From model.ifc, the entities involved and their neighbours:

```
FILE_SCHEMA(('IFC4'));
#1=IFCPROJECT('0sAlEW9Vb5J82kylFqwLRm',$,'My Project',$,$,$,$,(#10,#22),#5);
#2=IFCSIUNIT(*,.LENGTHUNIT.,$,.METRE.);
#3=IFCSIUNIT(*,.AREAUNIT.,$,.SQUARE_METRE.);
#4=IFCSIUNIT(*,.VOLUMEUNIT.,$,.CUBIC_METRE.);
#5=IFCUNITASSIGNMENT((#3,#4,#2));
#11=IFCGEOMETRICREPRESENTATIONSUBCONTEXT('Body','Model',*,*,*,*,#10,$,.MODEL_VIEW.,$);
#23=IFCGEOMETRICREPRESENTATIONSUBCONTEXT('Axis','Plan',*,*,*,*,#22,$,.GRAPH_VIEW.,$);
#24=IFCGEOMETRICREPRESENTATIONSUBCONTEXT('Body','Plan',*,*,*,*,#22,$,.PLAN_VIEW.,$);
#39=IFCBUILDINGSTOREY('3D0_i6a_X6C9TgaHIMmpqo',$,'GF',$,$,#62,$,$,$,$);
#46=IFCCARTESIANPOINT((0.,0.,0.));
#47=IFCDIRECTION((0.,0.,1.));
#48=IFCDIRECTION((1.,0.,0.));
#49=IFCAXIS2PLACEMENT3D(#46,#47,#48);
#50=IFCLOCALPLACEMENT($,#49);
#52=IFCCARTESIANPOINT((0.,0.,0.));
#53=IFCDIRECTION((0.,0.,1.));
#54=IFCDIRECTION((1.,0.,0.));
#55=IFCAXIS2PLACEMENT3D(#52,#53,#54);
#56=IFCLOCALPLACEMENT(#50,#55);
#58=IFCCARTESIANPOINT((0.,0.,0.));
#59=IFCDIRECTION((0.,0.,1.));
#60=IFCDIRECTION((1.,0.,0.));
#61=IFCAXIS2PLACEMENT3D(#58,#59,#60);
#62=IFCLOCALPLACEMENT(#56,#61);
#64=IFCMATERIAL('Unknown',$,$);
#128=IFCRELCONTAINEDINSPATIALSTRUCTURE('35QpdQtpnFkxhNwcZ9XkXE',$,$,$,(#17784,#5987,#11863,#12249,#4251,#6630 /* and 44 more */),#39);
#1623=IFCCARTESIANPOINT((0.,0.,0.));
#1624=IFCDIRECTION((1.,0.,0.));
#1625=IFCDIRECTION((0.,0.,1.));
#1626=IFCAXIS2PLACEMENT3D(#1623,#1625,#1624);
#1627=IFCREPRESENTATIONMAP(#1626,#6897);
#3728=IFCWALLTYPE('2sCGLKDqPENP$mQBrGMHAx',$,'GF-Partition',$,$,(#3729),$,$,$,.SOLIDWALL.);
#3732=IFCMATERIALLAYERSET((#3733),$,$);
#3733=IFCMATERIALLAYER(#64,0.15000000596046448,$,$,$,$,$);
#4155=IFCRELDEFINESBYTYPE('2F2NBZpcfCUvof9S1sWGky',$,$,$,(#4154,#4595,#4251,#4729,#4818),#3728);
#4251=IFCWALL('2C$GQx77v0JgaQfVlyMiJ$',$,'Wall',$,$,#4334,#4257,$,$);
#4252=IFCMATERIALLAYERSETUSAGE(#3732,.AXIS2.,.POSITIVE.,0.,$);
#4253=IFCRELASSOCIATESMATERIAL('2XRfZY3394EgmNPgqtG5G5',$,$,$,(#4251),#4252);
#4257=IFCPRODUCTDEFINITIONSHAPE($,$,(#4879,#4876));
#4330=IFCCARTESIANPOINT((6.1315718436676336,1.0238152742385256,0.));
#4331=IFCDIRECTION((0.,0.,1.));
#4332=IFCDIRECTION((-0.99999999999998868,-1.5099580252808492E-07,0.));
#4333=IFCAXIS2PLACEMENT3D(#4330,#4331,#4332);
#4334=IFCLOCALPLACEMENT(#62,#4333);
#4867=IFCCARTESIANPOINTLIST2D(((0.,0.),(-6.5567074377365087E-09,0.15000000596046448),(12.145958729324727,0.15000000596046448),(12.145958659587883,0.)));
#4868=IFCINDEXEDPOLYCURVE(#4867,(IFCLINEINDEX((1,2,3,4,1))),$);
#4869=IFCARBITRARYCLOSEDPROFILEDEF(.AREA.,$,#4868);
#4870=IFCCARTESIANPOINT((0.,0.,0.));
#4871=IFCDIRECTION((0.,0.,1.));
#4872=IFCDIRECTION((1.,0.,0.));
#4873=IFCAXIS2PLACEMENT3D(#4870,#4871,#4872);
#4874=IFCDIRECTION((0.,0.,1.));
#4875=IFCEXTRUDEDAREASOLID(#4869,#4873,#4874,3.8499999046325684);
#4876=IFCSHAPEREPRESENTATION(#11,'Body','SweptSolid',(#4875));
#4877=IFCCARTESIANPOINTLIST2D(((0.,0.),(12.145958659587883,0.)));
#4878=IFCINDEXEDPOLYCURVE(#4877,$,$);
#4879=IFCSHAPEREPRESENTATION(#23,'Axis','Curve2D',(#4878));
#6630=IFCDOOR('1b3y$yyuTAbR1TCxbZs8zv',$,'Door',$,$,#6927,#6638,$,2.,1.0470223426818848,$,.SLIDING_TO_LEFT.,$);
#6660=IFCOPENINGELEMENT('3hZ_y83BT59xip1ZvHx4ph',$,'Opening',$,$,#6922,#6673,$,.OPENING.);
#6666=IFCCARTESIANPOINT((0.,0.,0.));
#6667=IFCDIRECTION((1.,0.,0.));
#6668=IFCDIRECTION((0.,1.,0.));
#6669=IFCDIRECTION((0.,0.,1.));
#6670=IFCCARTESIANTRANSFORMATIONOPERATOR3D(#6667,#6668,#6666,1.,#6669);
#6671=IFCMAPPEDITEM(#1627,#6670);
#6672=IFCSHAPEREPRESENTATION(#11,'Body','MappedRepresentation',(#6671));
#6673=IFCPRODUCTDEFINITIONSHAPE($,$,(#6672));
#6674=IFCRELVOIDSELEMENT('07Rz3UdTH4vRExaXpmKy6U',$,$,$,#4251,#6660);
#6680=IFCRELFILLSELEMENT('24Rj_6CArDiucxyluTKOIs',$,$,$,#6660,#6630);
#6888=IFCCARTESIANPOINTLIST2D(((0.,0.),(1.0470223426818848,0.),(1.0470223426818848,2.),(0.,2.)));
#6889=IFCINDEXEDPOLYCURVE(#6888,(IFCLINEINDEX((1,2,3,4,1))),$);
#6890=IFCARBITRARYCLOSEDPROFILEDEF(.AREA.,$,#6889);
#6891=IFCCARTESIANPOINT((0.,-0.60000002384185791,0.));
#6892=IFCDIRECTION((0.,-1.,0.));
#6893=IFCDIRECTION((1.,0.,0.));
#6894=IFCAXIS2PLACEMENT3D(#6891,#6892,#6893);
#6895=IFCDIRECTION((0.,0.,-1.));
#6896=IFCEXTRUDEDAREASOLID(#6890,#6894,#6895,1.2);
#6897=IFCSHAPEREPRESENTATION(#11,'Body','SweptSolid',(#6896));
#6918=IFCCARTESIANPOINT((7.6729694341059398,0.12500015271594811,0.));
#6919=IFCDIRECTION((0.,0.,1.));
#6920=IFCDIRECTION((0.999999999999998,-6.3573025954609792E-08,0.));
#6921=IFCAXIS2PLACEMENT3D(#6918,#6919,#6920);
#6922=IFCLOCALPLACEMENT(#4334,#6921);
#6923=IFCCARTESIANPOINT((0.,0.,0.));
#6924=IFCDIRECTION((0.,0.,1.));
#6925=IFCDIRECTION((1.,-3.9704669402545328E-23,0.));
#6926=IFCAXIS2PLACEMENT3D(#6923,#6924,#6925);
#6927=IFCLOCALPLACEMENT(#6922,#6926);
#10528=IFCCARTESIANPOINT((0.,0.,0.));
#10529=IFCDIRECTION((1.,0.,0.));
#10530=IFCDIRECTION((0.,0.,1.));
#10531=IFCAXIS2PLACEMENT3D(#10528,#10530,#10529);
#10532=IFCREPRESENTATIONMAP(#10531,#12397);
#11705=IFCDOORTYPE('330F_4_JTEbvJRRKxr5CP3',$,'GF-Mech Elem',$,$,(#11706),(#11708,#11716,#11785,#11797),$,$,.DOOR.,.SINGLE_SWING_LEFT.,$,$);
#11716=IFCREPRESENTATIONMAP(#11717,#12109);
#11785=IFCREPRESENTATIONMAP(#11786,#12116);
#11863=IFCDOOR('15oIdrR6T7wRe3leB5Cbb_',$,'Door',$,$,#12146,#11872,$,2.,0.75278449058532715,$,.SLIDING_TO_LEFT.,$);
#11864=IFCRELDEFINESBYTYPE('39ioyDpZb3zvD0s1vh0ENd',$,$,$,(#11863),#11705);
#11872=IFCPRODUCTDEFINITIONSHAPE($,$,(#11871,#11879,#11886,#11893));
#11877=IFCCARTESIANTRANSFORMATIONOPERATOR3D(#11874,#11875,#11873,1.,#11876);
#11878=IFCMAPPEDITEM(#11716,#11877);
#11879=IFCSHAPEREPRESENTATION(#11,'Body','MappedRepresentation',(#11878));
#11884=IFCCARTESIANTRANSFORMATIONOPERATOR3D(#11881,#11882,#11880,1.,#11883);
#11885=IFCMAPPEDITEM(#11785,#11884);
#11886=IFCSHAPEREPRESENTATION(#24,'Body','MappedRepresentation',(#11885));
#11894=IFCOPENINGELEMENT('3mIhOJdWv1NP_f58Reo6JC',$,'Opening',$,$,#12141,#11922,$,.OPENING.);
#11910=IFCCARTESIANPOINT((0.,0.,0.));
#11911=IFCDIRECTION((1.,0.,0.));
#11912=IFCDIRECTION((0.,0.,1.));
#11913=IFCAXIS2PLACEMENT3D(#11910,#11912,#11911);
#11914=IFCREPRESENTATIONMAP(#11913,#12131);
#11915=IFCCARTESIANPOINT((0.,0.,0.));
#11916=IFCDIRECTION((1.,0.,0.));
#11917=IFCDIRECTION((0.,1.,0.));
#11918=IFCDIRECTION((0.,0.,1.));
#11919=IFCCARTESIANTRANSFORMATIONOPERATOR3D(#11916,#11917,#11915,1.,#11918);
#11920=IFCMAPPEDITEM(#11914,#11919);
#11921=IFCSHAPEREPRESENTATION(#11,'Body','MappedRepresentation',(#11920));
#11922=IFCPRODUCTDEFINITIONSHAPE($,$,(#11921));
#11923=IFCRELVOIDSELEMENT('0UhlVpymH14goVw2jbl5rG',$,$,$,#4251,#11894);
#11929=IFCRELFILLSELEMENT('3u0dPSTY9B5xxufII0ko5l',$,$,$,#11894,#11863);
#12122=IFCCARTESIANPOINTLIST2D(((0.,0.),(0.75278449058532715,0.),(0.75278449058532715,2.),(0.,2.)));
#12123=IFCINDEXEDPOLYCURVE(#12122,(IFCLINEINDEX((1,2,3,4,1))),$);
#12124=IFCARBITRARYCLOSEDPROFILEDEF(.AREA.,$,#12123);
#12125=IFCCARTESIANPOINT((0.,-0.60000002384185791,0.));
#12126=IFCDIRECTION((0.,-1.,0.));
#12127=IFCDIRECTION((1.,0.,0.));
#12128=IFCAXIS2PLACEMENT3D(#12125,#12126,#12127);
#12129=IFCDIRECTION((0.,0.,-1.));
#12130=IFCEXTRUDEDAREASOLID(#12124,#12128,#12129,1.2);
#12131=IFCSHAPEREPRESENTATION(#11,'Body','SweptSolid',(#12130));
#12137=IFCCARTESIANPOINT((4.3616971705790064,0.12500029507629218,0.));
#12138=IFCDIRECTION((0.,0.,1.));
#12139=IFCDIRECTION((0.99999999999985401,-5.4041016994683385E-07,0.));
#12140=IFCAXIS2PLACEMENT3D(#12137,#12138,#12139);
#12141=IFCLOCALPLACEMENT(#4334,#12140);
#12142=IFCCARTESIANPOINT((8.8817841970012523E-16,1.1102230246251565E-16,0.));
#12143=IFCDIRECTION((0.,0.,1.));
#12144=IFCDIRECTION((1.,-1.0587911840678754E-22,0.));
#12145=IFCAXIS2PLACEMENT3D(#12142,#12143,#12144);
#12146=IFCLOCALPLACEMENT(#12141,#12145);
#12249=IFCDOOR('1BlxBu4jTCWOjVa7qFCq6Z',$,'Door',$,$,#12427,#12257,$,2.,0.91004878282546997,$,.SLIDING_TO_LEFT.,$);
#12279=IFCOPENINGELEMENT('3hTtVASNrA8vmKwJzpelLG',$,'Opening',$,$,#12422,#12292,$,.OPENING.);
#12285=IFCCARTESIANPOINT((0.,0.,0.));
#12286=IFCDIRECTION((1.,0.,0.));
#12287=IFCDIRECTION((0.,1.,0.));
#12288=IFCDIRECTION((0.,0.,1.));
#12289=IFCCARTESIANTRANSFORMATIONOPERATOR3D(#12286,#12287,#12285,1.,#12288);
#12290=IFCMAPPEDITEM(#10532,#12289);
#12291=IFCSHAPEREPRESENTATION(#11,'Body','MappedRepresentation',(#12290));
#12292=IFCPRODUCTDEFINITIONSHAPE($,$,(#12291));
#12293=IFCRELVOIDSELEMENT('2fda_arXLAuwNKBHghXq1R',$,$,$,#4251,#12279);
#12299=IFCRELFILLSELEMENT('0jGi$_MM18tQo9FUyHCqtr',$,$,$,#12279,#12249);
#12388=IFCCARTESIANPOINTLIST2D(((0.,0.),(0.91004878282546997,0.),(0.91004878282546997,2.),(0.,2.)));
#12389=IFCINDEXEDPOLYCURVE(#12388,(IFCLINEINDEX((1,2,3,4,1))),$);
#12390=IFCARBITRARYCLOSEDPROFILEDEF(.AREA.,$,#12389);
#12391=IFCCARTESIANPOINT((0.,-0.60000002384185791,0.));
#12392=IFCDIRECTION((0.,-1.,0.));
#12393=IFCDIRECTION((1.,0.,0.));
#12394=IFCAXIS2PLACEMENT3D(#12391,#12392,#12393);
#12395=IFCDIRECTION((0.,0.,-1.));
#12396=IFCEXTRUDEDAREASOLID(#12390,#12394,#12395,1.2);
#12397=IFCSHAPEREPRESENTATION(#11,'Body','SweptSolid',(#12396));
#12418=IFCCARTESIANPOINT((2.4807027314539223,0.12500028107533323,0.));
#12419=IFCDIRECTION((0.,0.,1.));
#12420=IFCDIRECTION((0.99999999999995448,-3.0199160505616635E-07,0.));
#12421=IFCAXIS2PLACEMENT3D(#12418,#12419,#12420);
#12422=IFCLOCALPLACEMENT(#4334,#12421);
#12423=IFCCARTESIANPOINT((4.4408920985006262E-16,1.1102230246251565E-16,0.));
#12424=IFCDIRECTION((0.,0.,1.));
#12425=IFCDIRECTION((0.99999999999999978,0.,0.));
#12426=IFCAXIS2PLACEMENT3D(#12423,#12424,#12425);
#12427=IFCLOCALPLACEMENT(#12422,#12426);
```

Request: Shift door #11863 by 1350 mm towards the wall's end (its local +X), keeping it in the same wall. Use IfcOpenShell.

```python
import ifcopenshell
import ifcopenshell.api.geometry
import ifcopenshell.util.placement

model = ifcopenshell.open("model.ifc")

door = model.by_guid("15oIdrR6T7wRe3leB5Cbb_")
opening = door.FillsVoids[0].RelatingOpeningElement
wall = opening.VoidsElements[0].RelatingBuildingElement

wall_matrix = ifcopenshell.util.placement.get_local_placement(wall.ObjectPlacement)
shift = wall_matrix[:3, 0] * 1.35
before = ifcopenshell.util.placement.get_local_placement(door.ObjectPlacement)[:3, 3].copy()

# The door is placed relative to its opening, so it follows when the opening moves.
matrix = ifcopenshell.util.placement.get_local_placement(opening.ObjectPlacement)
matrix[:3, 3] += shift
ifcopenshell.api.geometry.edit_object_placement(
    model, product=opening, matrix=matrix, is_si=False, should_transform_children=True
)

after = ifcopenshell.util.placement.get_local_placement(door.ObjectPlacement)[:3, 3]
print("door moved by", (after - before).round(3) + 0.0)

model.write("model_rev.ifc")
```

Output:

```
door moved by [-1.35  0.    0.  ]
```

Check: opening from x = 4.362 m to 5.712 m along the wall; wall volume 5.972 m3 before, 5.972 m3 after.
